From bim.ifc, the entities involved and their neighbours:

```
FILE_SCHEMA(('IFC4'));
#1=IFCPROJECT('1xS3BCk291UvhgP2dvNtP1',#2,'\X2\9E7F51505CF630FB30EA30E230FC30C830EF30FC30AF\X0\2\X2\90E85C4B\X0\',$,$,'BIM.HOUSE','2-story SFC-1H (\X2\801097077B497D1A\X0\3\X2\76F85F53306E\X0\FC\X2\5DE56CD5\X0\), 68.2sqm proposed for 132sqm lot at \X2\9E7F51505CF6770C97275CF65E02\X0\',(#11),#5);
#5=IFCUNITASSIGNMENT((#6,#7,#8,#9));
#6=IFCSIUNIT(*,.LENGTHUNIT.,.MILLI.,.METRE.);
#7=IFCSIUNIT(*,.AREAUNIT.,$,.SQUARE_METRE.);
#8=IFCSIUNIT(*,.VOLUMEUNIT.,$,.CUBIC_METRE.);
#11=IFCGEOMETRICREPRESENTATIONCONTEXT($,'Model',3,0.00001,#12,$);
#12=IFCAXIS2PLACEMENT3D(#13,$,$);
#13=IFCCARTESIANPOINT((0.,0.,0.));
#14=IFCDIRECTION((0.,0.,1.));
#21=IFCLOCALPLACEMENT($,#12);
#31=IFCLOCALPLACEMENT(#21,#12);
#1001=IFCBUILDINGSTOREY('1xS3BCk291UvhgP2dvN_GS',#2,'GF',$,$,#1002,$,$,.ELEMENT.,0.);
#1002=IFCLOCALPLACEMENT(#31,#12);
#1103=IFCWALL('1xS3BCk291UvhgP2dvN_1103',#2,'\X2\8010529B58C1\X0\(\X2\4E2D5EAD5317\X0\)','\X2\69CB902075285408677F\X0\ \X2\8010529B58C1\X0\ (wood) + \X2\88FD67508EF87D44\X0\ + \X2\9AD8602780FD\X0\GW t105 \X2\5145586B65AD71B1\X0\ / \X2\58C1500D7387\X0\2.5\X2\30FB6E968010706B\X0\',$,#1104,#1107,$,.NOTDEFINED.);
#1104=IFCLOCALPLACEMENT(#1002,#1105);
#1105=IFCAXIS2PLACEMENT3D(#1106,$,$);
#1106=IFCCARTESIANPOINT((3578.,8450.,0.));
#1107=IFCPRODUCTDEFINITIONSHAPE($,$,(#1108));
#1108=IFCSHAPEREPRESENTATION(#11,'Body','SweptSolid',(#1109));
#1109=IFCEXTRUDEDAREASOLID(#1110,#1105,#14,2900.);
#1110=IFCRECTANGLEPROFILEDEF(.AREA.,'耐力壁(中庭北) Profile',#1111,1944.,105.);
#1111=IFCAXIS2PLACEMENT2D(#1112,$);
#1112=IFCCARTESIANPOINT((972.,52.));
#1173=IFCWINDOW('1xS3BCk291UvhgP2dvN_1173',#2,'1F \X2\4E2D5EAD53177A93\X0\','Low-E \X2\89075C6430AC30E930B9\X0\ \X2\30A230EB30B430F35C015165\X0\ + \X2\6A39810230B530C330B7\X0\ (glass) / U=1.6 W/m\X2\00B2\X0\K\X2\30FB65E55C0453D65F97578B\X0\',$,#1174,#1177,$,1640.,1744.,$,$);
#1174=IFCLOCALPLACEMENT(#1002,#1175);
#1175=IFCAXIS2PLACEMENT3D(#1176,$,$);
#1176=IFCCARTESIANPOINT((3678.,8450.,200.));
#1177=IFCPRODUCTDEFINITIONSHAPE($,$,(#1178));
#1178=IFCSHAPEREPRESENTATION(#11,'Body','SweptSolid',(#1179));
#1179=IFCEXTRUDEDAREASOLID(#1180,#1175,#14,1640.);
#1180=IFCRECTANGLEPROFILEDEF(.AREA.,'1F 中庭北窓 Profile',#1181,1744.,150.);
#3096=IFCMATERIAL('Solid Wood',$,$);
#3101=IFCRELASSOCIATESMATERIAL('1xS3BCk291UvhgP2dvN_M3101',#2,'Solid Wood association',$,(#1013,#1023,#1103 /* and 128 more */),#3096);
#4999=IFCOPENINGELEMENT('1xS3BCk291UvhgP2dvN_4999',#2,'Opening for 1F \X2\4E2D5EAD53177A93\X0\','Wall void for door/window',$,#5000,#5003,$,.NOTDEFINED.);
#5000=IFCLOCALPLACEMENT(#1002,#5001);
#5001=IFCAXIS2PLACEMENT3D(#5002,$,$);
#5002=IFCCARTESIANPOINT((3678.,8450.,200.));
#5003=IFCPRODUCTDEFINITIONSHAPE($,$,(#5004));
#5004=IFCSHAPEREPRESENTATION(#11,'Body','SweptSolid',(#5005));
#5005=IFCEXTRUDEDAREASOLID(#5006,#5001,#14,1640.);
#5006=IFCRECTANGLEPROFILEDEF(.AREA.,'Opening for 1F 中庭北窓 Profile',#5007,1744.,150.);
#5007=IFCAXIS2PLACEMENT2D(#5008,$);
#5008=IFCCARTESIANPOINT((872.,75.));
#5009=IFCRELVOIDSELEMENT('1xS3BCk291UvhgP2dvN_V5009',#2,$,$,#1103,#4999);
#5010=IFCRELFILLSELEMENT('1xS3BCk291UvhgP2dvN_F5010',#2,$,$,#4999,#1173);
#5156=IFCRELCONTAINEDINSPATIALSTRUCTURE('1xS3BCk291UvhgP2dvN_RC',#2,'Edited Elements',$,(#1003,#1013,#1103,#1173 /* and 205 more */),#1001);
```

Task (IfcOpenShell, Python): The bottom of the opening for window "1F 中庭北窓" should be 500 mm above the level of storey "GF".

```python
import numpy as np
import ifcopenshell
import ifcopenshell.api.geometry
import ifcopenshell.geom
import ifcopenshell.util.element
import ifcopenshell.util.placement
import ifcopenshell.util.shape
import ifcopenshell.util.unit

model = ifcopenshell.open("bim.ifc")
unit_scale = ifcopenshell.util.unit.calculate_unit_scale(model)

window = model.by_guid("1xS3BCk291UvhgP2dvN_1173")
opening = window.FillsVoids[0].RelatingOpeningElement
storey = ifcopenshell.util.element.get_container(window, ifc_class="IfcBuildingStorey")
level = ifcopenshell.util.placement.get_local_placement(storey.ObjectPlacement)[2, 3]

# The opening's origin need not be at the sill, so measure its lowest point.
shape = ifcopenshell.geom.create_shape(ifcopenshell.geom.settings(), opening)
bottom = ifcopenshell.util.shape.get_shape_bottom_elevation(shape, shape.geometry) / unit_scale
dz = level + 500.0 - bottom

shift = np.array([0.0, 0.0, dz])
# The window is not placed relative to its opening, so move both.
for product in (opening, window):
    matrix = ifcopenshell.util.placement.get_local_placement(product.ObjectPlacement)
    matrix[:3, 3] += shift
    ifcopenshell.api.geometry.edit_object_placement(model, product=product, matrix=matrix, is_si=False)

print(f"moved by {dz * unit_scale:+.3f} m")

model.write("bim_v2.ifc")
```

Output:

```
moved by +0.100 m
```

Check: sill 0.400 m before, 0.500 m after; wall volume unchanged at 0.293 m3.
